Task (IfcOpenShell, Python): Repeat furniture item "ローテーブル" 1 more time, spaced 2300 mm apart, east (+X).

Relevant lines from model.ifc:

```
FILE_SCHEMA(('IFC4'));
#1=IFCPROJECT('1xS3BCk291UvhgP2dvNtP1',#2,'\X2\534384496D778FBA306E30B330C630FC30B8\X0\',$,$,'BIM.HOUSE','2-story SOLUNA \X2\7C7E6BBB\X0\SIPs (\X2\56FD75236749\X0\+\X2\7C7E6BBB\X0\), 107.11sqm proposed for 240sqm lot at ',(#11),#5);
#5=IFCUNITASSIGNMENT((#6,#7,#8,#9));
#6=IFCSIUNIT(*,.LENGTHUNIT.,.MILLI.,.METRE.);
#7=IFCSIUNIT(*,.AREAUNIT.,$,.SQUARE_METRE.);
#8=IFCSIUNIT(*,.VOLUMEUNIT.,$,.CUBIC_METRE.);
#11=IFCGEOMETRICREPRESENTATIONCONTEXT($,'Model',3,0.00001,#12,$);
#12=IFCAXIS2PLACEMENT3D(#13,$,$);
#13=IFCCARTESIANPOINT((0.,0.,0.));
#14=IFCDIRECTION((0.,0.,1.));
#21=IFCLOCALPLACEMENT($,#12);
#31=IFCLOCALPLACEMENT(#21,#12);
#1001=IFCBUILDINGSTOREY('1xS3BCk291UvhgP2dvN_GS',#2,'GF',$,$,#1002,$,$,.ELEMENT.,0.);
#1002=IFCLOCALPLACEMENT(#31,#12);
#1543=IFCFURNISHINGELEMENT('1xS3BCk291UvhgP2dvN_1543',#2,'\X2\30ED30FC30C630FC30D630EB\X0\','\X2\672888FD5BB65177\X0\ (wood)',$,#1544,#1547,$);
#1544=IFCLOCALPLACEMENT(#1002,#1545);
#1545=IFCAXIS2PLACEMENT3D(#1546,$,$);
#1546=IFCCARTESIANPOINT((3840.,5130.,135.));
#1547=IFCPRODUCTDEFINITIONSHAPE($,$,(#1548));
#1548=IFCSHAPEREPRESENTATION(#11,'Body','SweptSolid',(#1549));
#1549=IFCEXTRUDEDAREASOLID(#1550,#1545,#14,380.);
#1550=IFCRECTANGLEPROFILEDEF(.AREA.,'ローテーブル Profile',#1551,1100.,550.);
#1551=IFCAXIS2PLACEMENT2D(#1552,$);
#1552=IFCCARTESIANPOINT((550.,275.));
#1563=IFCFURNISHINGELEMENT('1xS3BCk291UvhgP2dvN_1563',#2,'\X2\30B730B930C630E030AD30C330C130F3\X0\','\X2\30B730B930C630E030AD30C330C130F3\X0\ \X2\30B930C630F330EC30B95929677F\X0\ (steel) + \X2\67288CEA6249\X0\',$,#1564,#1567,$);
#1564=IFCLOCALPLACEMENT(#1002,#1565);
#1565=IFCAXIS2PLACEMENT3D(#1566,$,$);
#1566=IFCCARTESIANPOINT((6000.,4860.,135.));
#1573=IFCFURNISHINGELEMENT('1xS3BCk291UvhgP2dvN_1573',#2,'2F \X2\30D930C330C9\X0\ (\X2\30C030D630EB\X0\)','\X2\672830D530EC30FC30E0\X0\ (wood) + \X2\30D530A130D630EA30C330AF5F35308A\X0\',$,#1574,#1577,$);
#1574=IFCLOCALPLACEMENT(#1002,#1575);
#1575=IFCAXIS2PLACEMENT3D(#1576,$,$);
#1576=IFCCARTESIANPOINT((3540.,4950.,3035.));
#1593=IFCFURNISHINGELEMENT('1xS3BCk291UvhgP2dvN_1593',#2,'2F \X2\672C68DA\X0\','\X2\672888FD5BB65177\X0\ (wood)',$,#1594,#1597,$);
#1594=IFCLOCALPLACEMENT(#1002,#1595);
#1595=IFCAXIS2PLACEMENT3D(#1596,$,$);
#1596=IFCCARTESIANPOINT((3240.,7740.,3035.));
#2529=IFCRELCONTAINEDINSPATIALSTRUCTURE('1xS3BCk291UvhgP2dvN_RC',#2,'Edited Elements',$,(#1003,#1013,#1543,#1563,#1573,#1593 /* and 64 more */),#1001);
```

```python
import numpy as np
import ifcopenshell
import ifcopenshell.api.geometry
import ifcopenshell.api.root
import ifcopenshell.util.element
import ifcopenshell.util.placement
import ifcopenshell.util.unit

model = ifcopenshell.open("model.ifc")
unit_scale = ifcopenshell.util.unit.calculate_unit_scale(model)


def reuse_history(source, copy):
    """copy_class also copies each property set's owner history, people and application; keep the originals."""
    for rel in copy.IsDefinedBy:
        if rel.is_a("IfcRelDefinesByProperties") and (history := rel.RelatingPropertyDefinition.OwnerHistory):
            rel.RelatingPropertyDefinition.OwnerHistory = source.OwnerHistory
            ifcopenshell.util.element.remove_deep2(model, history)


source = model.by_id(1543)
base = ifcopenshell.util.placement.get_local_placement(source.ObjectPlacement)
step = np.array([1.0, 0.0, 0.0]) * 2.3 / unit_scale

for i in range(1, 2):
    copy = ifcopenshell.api.root.copy_class(model, product=source)
    copy.Representation = ifcopenshell.util.element.copy_deep(
        model, source.Representation, exclude=["IfcGeometricRepresentationContext", "IfcRepresentationMap"]
    )
    reuse_history(source, copy)
    matrix = base.copy()
    matrix[:3, 3] += i * step
    print("added at", matrix[:3, 3].round(3) + 0.0)
    ifcopenshell.api.geometry.edit_object_placement(model, product=copy, matrix=matrix, is_si=False)

model.write("model_edited.ifc")
```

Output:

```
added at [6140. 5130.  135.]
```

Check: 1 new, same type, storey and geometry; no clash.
